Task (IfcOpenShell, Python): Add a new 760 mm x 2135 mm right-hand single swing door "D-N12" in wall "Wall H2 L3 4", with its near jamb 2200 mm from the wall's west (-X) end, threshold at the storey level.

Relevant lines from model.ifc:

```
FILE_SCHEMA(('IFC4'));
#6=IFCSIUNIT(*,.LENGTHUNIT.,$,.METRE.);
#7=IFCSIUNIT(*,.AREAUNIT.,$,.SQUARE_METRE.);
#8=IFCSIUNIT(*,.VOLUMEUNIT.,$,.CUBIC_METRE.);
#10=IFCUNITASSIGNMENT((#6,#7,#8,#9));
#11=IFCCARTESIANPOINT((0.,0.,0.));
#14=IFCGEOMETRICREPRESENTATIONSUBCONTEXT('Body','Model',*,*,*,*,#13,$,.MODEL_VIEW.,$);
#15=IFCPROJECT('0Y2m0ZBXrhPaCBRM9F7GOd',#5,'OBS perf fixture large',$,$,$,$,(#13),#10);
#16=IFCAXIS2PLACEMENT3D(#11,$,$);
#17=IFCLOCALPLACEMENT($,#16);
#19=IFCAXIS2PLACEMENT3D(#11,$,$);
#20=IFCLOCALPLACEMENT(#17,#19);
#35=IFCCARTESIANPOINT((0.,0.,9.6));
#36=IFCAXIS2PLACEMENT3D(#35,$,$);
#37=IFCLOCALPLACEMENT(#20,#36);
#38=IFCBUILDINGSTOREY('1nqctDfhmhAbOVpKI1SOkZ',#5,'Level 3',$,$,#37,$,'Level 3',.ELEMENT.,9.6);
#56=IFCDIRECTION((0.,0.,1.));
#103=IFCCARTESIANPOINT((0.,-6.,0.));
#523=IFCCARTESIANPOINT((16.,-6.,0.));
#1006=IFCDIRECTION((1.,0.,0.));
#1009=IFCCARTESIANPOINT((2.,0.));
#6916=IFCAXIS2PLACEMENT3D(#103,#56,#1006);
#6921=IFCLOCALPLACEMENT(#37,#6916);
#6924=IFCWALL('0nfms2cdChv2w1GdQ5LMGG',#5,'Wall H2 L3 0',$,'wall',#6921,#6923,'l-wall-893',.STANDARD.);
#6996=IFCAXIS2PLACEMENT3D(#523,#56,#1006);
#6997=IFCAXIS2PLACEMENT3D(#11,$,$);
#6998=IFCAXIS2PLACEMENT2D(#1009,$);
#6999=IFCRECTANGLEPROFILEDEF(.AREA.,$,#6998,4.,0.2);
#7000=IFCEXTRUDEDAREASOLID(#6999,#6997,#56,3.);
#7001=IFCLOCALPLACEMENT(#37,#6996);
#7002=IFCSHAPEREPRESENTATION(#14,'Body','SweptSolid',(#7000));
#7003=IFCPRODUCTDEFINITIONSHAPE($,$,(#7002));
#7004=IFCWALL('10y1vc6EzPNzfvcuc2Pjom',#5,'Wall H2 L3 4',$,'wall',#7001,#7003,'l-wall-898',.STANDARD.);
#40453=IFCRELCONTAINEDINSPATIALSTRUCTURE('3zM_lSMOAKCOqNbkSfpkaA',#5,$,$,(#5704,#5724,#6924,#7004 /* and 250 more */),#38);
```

```python
import numpy as np
import ifcopenshell
import ifcopenshell.api.feature
import ifcopenshell.api.geometry
import ifcopenshell.api.root
import ifcopenshell.api.spatial
import ifcopenshell.geom
import ifcopenshell.util.element
import ifcopenshell.util.placement
import ifcopenshell.util.representation
import ifcopenshell.util.shape
import ifcopenshell.util.unit

model = ifcopenshell.open("model.ifc")
unit_scale = ifcopenshell.util.unit.calculate_unit_scale(model)
settings = ifcopenshell.geom.settings()


def volume(element):
    """Net volume in cubic metres, openings subtracted."""
    shape = ifcopenshell.geom.create_shape(settings, element)
    return ifcopenshell.util.shape.get_volume(shape.geometry)


wall = model.by_guid("10y1vc6EzPNzfvcuc2Pjom")
storey = ifcopenshell.util.element.get_container(wall, ifc_class="IfcBuildingStorey")
context = ifcopenshell.util.representation.get_context(model, "Model", "Body", "MODEL_VIEW")
before = volume(wall)

width, height, from_end, sill = 0.76, 2.135, 2.2, 0.0  # metres

# The wall runs along its own X axis, and the end named is its -X end.
wall_shape = ifcopenshell.geom.create_shape(settings, wall)
x, y, z = ifcopenshell.util.shape.get_vertices(wall_shape.geometry).T
start = x.min() + from_end
face, thickness = float(y.min()), float(y.max() - y.min())
wall_matrix = ifcopenshell.util.placement.get_local_placement(wall.ObjectPlacement)
level = ifcopenshell.util.placement.get_local_placement(storey.ObjectPlacement)[2, 3]


def in_wall(x, y):
    """Placement at x, y metres in the wall's axes, at sill height."""
    matrix = wall_matrix.copy()
    matrix[:, 3] = wall_matrix @ np.array([x / unit_scale, y / unit_scale, 0.0, 1.0])
    matrix[2, 3] = level + sill / unit_scale
    return matrix


# Opening: a box that overshoots both wall faces by 50 mm.
opening = ifcopenshell.api.root.create_entity(model, ifc_class="IfcOpeningElement", predefined_type="OPENING")
box = ifcopenshell.api.geometry.add_wall_representation(
    model, context=context, length=width, height=height, thickness=thickness + 0.1
)
ifcopenshell.api.geometry.assign_representation(model, product=opening, representation=box)
ifcopenshell.api.geometry.edit_object_placement(model, product=opening, matrix=in_wall(start, face - 0.05), is_si=False)
ifcopenshell.api.feature.add_feature(model, feature=opening, element=wall)

door = ifcopenshell.api.root.create_entity(model, ifc_class="IfcDoor", name="D-N12", predefined_type="DOOR")
door.OverallWidth, door.OverallHeight = width / unit_scale, height / unit_scale
door.OperationType = "SINGLE_SWING_RIGHT"
body = ifcopenshell.api.geometry.add_door_representation(
    model,
    context=context,
    overall_width=door.OverallWidth,
    overall_height=door.OverallHeight,
    operation_type="SINGLE_SWING_RIGHT",
    lining_properties={"LiningDepth": thickness / unit_scale, "ThresholdDepth": thickness / unit_scale},
)
ifcopenshell.api.geometry.assign_representation(model, product=door, representation=body)
ifcopenshell.api.spatial.assign_container(model, products=[door], relating_structure=storey)
ifcopenshell.api.feature.add_filling(model, opening=opening, element=door)

# The lining spans the wall, so the door starts at the wall face.
ifcopenshell.api.geometry.edit_object_placement(model, product=door, matrix=in_wall(start, face), is_si=False)

after = volume(wall)

print(f"wall volume {before:.3f} -> {after:.3f} m3")

model.write("model_edited.ifc")
```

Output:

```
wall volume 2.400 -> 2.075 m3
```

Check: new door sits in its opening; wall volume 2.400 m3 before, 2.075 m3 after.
